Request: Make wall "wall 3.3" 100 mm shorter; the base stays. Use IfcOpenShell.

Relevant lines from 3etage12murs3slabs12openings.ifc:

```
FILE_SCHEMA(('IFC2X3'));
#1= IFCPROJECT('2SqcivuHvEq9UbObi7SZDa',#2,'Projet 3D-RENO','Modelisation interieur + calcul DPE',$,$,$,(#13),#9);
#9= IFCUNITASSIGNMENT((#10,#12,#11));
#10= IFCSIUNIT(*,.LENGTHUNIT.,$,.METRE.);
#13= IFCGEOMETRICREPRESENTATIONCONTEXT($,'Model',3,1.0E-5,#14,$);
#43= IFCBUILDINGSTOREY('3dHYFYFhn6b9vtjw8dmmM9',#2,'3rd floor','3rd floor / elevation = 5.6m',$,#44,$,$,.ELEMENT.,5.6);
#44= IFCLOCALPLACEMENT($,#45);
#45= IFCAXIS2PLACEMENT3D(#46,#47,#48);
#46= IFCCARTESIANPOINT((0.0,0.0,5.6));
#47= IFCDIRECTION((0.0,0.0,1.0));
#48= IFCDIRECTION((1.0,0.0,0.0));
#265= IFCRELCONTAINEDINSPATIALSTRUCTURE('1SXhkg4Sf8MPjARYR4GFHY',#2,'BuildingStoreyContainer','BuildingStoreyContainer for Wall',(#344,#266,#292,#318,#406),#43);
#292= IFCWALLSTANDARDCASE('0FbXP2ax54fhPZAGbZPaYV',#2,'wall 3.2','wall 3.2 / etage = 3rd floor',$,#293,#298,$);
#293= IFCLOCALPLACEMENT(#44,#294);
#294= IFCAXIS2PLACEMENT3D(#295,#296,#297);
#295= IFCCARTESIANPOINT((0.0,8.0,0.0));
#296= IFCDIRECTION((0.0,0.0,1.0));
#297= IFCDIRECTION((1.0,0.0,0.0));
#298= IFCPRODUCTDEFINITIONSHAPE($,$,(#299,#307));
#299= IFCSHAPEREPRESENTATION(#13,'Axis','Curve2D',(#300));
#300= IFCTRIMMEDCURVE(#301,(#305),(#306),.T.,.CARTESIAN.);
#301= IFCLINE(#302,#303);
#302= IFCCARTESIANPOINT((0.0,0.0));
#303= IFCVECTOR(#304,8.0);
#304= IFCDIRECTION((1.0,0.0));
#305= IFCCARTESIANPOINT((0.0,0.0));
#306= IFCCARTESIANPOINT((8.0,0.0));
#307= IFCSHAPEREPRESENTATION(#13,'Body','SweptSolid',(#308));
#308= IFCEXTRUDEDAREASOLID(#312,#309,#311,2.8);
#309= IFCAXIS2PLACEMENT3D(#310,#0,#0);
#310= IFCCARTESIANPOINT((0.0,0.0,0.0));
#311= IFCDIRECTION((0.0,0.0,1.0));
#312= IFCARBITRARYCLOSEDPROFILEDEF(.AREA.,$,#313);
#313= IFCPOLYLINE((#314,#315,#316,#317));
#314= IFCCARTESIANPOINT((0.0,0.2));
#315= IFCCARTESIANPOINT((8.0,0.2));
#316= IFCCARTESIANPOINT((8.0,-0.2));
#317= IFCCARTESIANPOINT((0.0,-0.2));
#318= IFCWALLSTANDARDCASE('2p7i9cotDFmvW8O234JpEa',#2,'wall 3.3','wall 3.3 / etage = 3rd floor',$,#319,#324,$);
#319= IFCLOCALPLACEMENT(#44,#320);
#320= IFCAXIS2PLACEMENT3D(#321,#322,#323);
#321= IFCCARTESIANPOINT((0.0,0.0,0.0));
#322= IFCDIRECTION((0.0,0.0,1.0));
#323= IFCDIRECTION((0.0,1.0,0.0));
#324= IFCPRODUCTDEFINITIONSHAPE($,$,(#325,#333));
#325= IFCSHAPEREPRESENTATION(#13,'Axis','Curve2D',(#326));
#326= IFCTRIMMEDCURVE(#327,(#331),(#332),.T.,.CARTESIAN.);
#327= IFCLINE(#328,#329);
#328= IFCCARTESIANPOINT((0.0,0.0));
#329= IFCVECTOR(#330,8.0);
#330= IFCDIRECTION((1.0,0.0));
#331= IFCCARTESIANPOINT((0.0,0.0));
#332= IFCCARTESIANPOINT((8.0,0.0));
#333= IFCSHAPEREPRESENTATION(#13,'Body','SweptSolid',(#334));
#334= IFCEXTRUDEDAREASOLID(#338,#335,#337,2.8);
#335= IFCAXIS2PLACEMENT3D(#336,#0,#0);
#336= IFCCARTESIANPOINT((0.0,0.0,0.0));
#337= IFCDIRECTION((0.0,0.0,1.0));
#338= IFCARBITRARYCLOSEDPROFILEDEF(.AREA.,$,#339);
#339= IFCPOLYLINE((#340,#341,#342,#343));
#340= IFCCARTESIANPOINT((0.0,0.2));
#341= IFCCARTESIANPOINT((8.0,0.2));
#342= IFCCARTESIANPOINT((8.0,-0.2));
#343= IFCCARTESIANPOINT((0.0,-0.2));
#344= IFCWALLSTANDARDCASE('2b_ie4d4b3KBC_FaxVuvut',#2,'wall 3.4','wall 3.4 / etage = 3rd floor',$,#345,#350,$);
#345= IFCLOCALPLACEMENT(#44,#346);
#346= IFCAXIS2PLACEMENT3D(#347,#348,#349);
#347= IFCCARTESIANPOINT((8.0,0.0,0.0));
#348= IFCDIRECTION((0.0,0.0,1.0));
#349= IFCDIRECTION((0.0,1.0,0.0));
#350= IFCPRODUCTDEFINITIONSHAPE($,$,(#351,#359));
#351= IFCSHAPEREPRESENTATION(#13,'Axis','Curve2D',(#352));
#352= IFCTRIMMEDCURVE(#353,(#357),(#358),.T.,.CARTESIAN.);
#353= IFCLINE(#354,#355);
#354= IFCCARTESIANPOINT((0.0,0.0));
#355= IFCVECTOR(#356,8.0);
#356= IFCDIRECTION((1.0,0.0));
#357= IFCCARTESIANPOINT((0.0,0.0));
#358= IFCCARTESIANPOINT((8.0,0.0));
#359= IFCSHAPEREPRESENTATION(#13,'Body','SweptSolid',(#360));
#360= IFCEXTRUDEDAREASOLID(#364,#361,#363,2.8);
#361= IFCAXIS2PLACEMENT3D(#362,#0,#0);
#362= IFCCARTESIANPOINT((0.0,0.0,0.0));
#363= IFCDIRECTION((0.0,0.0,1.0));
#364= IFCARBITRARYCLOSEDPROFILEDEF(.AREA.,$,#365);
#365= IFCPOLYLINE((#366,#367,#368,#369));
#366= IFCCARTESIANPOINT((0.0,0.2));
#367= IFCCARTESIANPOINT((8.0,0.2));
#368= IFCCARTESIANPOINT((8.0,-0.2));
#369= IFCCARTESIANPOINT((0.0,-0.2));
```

```python
import ifcopenshell
import ifcopenshell.geom
import ifcopenshell.util.shape
import ifcopenshell.util.unit

model = ifcopenshell.open("3etage12murs3slabs12openings.ifc")
unit_scale = ifcopenshell.util.unit.calculate_unit_scale(model)
settings = ifcopenshell.geom.settings()


def volume(element):
    """Net volume in cubic metres, openings subtracted."""
    shape = ifcopenshell.geom.create_shape(settings, element)
    return ifcopenshell.util.shape.get_volume(shape.geometry)


wall = model.by_guid("2p7i9cotDFmvW8O234JpEa")
before = volume(wall)

body = next(r for r in wall.Representation.Representations if r.RepresentationIdentifier == "Body")
solid = body.Items[0]
old_height = solid.Depth
solid.Depth -= 0.1 / unit_scale
after = volume(wall)

print(f"height {old_height:g} -> {solid.Depth:g}, volume {before:.3f} -> {after:.3f} m3")

model.write("3etage12murs3slabs12openings_updated.ifc")
```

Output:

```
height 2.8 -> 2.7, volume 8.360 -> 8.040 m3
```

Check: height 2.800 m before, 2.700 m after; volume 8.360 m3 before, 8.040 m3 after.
